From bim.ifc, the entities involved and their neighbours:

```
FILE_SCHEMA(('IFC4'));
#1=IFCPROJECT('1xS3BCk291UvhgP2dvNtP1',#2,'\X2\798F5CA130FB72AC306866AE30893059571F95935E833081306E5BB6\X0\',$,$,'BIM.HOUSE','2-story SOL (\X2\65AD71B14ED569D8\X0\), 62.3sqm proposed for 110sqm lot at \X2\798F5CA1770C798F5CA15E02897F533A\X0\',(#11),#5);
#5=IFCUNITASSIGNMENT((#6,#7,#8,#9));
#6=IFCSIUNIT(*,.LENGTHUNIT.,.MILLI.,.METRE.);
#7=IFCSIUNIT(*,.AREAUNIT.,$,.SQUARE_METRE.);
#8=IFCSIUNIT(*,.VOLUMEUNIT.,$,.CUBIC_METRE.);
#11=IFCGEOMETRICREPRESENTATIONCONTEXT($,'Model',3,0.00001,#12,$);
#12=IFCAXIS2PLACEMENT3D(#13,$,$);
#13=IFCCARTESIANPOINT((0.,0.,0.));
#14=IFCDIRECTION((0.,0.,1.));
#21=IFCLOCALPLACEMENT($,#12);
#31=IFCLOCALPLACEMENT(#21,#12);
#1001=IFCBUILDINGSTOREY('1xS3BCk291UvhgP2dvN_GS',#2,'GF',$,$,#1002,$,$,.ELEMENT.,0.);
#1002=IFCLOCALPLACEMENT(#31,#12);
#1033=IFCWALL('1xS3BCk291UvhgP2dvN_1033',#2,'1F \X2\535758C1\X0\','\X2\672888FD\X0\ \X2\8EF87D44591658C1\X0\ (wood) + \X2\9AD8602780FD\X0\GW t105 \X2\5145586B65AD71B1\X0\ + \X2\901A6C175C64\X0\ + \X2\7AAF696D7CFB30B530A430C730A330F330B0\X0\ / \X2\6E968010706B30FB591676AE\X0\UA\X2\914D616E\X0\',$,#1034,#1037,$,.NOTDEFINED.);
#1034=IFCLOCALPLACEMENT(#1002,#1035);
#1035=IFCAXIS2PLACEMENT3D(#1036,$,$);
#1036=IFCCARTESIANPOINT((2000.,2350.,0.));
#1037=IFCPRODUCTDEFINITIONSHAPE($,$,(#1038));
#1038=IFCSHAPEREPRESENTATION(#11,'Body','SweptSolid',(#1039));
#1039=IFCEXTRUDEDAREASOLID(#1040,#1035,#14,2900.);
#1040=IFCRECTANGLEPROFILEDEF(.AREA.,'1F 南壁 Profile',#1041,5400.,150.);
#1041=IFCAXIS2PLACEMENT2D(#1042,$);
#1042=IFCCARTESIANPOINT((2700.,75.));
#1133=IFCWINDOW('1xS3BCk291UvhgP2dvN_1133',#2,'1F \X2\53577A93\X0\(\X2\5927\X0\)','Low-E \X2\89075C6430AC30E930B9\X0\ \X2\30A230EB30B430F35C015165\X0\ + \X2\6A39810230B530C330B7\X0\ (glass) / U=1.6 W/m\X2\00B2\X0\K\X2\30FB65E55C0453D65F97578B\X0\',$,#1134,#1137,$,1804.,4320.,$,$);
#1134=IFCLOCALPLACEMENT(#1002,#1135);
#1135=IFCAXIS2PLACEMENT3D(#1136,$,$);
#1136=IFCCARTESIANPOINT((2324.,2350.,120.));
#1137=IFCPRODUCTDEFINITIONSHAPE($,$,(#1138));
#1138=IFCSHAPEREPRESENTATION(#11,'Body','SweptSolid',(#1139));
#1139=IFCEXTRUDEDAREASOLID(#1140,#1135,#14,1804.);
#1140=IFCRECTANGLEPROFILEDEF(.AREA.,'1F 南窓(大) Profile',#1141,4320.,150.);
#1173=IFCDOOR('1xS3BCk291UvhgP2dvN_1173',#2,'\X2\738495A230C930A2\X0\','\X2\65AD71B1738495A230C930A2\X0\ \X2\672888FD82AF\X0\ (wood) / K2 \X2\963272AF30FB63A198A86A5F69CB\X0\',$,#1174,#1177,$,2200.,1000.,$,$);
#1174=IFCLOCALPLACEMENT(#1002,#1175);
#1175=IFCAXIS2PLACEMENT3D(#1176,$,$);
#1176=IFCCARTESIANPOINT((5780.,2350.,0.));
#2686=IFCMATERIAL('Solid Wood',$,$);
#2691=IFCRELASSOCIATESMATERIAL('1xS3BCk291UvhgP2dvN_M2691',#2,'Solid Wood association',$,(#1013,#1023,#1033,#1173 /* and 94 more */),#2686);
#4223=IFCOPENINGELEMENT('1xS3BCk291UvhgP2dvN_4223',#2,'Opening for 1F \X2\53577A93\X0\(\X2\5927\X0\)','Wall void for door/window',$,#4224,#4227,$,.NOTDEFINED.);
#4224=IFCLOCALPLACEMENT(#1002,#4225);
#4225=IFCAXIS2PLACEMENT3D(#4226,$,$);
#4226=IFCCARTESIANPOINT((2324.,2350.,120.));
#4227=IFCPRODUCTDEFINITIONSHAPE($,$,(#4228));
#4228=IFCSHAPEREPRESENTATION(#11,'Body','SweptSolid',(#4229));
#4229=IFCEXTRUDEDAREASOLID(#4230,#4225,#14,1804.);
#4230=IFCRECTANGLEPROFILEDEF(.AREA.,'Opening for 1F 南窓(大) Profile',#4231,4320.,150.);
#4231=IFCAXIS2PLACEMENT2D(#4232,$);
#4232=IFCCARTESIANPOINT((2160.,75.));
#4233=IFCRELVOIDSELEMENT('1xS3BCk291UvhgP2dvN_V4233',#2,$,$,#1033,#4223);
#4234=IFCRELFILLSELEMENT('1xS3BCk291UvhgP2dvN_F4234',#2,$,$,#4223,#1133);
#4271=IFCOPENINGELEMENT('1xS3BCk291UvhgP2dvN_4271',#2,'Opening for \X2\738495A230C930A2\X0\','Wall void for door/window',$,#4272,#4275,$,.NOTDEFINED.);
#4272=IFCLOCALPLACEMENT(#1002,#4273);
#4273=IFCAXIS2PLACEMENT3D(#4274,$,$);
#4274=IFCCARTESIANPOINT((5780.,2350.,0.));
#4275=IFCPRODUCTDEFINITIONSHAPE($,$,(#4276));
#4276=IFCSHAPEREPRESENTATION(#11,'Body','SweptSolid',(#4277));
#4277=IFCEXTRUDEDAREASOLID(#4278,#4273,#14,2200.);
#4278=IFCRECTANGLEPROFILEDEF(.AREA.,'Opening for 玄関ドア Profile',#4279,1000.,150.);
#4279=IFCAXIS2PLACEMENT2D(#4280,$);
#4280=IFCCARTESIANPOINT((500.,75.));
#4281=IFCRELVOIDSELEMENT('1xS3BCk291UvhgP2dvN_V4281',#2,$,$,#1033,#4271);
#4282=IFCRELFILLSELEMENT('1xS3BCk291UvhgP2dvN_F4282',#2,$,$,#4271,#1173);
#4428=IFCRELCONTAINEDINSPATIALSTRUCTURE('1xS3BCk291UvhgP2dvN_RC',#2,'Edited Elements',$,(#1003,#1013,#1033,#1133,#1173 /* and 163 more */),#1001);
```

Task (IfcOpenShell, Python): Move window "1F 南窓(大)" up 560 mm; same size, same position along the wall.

```python
import numpy as np
import ifcopenshell
import ifcopenshell.api.geometry
import ifcopenshell.util.placement
import ifcopenshell.util.unit

model = ifcopenshell.open("bim.ifc")
unit_scale = ifcopenshell.util.unit.calculate_unit_scale(model)

window = model.by_guid("1xS3BCk291UvhgP2dvN_1133")
opening = window.FillsVoids[0].RelatingOpeningElement
dz = 560.0

shift = np.array([0.0, 0.0, dz])
# The window is not placed relative to its opening, so move both.
for product in (opening, window):
    matrix = ifcopenshell.util.placement.get_local_placement(product.ObjectPlacement)
    matrix[:3, 3] += shift
    ifcopenshell.api.geometry.edit_object_placement(model, product=product, matrix=matrix, is_si=False)

print(f"moved by {dz * unit_scale:+.3f} m")

model.write("bim_updated.ifc")
```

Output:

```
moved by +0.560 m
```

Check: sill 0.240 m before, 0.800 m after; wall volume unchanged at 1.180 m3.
